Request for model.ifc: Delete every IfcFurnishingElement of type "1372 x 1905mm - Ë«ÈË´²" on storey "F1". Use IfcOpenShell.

First a look at what the model holds.

```python
import ifcopenshell
import ifcopenshell.util.element

model = ifcopenshell.open("model.ifc")
print(model.schema)
storey = next(s for s in model.by_type("IfcBuildingStorey") if s.Name == "F1")
furniture = [e for e in ifcopenshell.util.element.get_decomposition(storey) if e.is_a("IfcFurnishingElement")]
seen = {}
for e in furniture:
    element_type = ifcopenshell.util.element.get_type(e)
    name = element_type.Name if element_type not in (None, e) else None
    seen[name] = seen.get(name, 0) + 1
for name, count in sorted(seen.items(), key=str):
    print(count, "x", name)
```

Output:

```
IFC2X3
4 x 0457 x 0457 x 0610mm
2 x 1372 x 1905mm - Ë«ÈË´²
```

```python
import ifcopenshell
import ifcopenshell.api.root
import ifcopenshell.util.element

model = ifcopenshell.open("model.ifc")

storey = next(s for s in model.by_type("IfcBuildingStorey") if s.Name == "F1")
furniture = [e for e in ifcopenshell.util.element.get_decomposition(storey) if e.is_a("IfcFurnishingElement")]
targets = [e for e in furniture if (t := ifcopenshell.util.element.get_type(e)) not in (None, e) and t.Name == "1372 x 1905mm - Ë«ÈË´²"]

for e in targets:
    ifcopenshell.api.root.remove_product(model, product=e)
print(len(targets), "removed")

model.write("model_updated.ifc")
```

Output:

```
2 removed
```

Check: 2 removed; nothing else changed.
